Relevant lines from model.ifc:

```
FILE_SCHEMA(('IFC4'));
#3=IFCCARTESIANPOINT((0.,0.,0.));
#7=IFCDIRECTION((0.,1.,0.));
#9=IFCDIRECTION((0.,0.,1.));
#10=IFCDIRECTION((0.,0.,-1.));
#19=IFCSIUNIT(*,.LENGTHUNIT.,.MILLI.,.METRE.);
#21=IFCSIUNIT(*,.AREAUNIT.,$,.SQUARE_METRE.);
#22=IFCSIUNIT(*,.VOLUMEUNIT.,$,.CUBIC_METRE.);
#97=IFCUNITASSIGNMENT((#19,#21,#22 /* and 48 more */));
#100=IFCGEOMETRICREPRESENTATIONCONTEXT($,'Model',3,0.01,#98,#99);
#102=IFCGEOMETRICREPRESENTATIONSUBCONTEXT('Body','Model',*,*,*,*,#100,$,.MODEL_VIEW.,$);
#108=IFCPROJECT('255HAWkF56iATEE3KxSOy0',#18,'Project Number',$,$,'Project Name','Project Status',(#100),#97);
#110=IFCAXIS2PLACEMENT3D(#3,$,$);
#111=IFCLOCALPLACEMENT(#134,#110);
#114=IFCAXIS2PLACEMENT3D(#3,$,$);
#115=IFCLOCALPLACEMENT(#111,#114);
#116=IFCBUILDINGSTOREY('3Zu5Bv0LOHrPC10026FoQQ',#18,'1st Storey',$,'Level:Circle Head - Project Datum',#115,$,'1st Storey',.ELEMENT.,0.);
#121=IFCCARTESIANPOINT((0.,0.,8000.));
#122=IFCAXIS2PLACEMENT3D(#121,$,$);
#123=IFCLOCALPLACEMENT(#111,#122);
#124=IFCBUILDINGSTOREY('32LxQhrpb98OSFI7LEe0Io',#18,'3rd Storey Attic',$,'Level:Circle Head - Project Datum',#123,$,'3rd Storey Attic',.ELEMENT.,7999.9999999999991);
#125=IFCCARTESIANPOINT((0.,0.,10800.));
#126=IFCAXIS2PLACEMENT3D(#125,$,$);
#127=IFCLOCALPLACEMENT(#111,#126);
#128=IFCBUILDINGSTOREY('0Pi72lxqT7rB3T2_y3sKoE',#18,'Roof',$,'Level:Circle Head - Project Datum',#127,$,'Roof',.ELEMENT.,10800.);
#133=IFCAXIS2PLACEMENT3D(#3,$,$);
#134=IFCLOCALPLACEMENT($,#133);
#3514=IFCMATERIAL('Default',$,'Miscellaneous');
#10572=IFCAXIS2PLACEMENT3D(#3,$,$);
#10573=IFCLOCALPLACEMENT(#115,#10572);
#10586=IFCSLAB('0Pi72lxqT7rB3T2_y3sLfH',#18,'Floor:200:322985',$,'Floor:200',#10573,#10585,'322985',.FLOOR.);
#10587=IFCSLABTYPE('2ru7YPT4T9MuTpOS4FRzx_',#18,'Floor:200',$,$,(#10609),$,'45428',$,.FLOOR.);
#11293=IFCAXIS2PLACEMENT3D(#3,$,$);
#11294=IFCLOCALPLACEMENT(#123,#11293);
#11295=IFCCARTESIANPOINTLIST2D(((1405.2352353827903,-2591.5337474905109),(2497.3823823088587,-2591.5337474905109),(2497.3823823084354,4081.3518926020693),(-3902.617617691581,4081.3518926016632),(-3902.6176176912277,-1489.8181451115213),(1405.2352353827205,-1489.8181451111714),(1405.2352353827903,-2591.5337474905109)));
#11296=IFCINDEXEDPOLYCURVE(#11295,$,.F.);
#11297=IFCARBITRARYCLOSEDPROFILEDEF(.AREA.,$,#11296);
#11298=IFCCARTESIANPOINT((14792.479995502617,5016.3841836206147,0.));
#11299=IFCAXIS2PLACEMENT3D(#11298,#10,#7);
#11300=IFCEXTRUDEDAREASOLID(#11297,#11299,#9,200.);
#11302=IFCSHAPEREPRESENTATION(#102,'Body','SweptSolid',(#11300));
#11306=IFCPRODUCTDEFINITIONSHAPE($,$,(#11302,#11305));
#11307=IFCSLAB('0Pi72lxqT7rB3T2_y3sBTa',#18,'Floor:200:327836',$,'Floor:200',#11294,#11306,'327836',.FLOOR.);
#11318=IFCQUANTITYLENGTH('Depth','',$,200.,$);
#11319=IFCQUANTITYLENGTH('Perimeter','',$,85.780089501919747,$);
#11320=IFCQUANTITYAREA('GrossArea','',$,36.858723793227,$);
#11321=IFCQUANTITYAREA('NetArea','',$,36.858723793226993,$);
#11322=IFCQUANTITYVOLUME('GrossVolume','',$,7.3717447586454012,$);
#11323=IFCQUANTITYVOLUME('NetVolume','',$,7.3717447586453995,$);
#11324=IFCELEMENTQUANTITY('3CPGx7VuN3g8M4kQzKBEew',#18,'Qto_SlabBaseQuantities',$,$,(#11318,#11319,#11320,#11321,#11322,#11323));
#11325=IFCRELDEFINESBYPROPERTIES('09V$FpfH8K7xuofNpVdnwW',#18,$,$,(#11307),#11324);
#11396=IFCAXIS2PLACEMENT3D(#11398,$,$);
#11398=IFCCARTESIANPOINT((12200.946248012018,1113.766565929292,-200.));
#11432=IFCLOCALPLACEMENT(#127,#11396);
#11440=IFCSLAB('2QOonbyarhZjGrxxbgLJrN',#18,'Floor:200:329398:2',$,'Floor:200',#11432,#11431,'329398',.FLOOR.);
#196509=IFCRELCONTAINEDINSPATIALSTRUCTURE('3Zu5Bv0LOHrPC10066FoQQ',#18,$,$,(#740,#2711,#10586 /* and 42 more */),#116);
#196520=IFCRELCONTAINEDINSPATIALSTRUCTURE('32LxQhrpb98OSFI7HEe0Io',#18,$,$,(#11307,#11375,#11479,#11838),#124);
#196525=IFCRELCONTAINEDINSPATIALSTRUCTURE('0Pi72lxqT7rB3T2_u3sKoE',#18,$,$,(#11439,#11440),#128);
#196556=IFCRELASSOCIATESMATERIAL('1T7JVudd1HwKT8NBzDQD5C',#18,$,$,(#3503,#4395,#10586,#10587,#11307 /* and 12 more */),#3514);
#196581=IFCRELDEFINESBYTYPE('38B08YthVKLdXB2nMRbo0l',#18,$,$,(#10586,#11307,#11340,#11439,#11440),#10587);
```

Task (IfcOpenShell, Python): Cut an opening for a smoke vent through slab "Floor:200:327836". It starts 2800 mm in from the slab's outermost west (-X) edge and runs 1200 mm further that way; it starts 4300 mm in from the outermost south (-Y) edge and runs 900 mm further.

```python
import numpy as np
import ifcopenshell
import ifcopenshell.api.feature
import ifcopenshell.api.geometry
import ifcopenshell.api.pset
import ifcopenshell.api.root
import ifcopenshell.geom
import ifcopenshell.util.element
import ifcopenshell.util.placement
import ifcopenshell.util.representation
import ifcopenshell.util.shape
import ifcopenshell.util.unit

model = ifcopenshell.open("model.ifc")
unit_scale = ifcopenshell.util.unit.calculate_unit_scale(model)
area_scale = ifcopenshell.util.unit.calculate_unit_scale(model, "AREAUNIT")
volume_scale = ifcopenshell.util.unit.calculate_unit_scale(model, "VOLUMEUNIT")
settings = ifcopenshell.geom.settings()


def volume(element):
    """Net volume in cubic metres, openings subtracted."""
    shape = ifcopenshell.geom.create_shape(settings, element)
    return ifcopenshell.util.shape.get_volume(shape.geometry)


slab = model.by_guid("0Pi72lxqT7rB3T2_y3sBTa")
before = volume(slab)

# Extent in the slab's own axes, in metres. The edges named are its -X and -Y sides.
slab_shape = ifcopenshell.geom.create_shape(settings, slab)
vertices = ifcopenshell.util.shape.get_vertices(slab_shape.geometry)
x_min, y_min, bottom = vertices.min(axis=0)
top = vertices[:, 2].max()

opening = ifcopenshell.api.root.create_entity(model, ifc_class="IfcOpeningElement", name="Smoke vent opening", predefined_type="OPENING")
context = ifcopenshell.util.representation.get_context(model, "Model", "Body", "MODEL_VIEW")
width, depth = 1.2, 0.9
outline = [(0.0, 0.0), (width, 0.0), (width, depth), (0.0, depth), (0.0, 0.0)]
# Overshoot both faces by 50 mm so the cut is clean.
shape = ifcopenshell.api.geometry.add_slab_representation(
    model, context=context, depth=top - bottom + 0.1, polyline=outline
)
ifcopenshell.api.geometry.assign_representation(model, product=opening, representation=shape)

matrix = ifcopenshell.util.placement.get_local_placement(slab.ObjectPlacement)
matrix[:, 3] = matrix @ np.append(np.array([x_min + 2.8, y_min + 4.3, bottom - 0.05]) / unit_scale, 1.0)
ifcopenshell.api.geometry.edit_object_placement(model, product=opening, matrix=matrix, is_si=False)
ifcopenshell.api.feature.add_feature(model, feature=opening, element=slab)

after = volume(slab)

# Update the slab's stored quantities.
qto = model.by_id(ifcopenshell.util.element.get_pset(slab, "Qto_SlabBaseQuantities", should_inherit=False)["id"])
ifcopenshell.api.pset.edit_qto(model, qto=qto, properties={
    "NetArea": after / (top - bottom) / area_scale,
    "NetVolume": after / volume_scale,
})

print(f"slab volume {before:.3f} -> {after:.3f} m3")

model.write("model_edited.ifc")
```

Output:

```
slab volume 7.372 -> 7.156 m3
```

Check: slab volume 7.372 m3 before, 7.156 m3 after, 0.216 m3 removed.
